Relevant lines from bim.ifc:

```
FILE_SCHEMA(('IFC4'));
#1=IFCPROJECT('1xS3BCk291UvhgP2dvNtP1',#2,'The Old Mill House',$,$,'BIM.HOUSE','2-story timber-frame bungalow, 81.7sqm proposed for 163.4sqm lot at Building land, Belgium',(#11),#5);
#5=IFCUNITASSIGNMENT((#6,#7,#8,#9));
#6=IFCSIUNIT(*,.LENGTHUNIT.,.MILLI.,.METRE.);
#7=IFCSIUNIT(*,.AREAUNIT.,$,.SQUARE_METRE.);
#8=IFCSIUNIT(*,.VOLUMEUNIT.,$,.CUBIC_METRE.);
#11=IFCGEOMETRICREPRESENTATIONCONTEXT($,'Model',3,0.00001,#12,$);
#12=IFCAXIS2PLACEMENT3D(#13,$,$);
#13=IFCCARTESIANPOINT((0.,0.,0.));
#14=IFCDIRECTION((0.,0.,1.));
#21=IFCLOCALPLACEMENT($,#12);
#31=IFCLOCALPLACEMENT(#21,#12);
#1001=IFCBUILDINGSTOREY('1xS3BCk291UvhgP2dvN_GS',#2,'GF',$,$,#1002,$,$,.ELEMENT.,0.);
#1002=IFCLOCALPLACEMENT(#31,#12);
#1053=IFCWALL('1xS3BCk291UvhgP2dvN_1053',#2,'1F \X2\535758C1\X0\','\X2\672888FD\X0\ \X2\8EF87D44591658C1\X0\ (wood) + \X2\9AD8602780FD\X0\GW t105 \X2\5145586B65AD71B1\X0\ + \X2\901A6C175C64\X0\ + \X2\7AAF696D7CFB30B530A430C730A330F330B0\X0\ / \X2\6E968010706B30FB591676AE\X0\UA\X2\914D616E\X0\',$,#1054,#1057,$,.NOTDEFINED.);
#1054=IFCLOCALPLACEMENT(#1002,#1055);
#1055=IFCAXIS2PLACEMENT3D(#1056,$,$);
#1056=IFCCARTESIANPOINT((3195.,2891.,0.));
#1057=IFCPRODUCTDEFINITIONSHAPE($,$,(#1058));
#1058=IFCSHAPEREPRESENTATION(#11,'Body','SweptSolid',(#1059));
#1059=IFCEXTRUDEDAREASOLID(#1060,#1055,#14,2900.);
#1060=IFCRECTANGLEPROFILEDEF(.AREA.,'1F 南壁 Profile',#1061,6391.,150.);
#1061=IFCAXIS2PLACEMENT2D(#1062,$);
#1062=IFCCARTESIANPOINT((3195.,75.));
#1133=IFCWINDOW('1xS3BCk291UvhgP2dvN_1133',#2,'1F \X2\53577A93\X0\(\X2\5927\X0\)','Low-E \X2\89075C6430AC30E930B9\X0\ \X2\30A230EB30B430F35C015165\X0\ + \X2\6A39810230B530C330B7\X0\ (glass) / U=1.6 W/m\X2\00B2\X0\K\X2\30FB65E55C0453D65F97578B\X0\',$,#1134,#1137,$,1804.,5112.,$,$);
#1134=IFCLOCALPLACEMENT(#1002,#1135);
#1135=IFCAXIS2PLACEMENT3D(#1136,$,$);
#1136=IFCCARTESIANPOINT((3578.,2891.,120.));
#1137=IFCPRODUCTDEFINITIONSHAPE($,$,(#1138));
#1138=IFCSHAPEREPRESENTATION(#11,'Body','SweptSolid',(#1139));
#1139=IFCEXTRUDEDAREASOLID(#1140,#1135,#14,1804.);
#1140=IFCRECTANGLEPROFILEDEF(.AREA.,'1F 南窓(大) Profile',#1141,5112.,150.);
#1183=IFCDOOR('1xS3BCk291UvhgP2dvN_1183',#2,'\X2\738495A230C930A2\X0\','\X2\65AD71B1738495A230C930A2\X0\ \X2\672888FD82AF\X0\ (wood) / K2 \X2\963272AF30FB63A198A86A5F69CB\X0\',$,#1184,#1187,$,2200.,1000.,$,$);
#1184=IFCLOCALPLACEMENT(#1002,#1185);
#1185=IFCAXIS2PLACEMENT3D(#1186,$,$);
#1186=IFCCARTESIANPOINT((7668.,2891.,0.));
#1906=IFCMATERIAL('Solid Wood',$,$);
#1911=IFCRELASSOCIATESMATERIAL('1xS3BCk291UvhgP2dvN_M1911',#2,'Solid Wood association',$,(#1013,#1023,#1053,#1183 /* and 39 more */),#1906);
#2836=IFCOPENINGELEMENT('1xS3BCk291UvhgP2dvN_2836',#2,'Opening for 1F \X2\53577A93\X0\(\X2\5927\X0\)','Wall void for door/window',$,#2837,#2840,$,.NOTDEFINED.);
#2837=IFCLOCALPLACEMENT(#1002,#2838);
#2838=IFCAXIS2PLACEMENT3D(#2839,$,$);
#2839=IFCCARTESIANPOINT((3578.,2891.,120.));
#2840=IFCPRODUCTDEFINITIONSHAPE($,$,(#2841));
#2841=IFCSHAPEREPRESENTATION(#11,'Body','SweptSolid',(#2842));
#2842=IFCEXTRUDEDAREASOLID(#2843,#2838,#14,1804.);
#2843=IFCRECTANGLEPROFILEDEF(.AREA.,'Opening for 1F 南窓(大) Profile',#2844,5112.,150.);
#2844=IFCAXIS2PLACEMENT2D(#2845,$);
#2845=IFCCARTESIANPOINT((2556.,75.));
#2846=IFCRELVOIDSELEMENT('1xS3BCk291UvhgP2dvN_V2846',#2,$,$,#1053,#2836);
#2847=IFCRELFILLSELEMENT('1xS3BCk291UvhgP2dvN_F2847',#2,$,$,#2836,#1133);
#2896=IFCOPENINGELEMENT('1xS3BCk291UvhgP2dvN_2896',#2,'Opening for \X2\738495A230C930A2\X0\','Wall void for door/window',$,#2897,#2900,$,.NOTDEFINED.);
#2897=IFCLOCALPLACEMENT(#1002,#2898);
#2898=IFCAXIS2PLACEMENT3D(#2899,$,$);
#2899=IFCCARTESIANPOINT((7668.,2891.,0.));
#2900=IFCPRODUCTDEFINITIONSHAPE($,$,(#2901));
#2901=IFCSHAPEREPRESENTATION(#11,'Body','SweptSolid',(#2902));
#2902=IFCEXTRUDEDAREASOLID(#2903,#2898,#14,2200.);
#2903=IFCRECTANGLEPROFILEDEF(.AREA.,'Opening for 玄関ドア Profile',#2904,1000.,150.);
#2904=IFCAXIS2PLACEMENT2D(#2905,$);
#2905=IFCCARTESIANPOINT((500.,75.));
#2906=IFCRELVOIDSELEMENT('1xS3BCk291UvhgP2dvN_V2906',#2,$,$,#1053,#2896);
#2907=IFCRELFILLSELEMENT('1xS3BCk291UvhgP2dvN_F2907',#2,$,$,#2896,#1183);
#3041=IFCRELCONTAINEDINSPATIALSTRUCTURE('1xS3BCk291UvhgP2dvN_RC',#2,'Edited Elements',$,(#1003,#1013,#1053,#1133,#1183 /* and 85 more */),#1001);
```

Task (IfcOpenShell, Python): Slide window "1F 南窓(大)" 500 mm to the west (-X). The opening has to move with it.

```python
import ifcopenshell
import ifcopenshell.api.geometry
import ifcopenshell.util.placement
import ifcopenshell.util.unit

model = ifcopenshell.open("bim.ifc")
unit_scale = ifcopenshell.util.unit.calculate_unit_scale(model)

window = model.by_id(1133)
opening = window.FillsVoids[0].RelatingOpeningElement
wall = opening.VoidsElements[0].RelatingBuildingElement

wall_matrix = ifcopenshell.util.placement.get_local_placement(wall.ObjectPlacement)
shift = wall_matrix[:3, 0] * -0.5 / unit_scale
before = ifcopenshell.util.placement.get_local_placement(window.ObjectPlacement)[:3, 3].copy()

# The window is not placed relative to its opening, so move both.
for product in (opening, window):
    matrix = ifcopenshell.util.placement.get_local_placement(product.ObjectPlacement)
    matrix[:3, 3] += shift
    ifcopenshell.api.geometry.edit_object_placement(model, product=product, matrix=matrix, is_si=False)

after = ifcopenshell.util.placement.get_local_placement(window.ObjectPlacement)[:3, 3]
print("window moved by", (after - before).round(3) + 0.0)

model.write("bim_v2.ifc")
```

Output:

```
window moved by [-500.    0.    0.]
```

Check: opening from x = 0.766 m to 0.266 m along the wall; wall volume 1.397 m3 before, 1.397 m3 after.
